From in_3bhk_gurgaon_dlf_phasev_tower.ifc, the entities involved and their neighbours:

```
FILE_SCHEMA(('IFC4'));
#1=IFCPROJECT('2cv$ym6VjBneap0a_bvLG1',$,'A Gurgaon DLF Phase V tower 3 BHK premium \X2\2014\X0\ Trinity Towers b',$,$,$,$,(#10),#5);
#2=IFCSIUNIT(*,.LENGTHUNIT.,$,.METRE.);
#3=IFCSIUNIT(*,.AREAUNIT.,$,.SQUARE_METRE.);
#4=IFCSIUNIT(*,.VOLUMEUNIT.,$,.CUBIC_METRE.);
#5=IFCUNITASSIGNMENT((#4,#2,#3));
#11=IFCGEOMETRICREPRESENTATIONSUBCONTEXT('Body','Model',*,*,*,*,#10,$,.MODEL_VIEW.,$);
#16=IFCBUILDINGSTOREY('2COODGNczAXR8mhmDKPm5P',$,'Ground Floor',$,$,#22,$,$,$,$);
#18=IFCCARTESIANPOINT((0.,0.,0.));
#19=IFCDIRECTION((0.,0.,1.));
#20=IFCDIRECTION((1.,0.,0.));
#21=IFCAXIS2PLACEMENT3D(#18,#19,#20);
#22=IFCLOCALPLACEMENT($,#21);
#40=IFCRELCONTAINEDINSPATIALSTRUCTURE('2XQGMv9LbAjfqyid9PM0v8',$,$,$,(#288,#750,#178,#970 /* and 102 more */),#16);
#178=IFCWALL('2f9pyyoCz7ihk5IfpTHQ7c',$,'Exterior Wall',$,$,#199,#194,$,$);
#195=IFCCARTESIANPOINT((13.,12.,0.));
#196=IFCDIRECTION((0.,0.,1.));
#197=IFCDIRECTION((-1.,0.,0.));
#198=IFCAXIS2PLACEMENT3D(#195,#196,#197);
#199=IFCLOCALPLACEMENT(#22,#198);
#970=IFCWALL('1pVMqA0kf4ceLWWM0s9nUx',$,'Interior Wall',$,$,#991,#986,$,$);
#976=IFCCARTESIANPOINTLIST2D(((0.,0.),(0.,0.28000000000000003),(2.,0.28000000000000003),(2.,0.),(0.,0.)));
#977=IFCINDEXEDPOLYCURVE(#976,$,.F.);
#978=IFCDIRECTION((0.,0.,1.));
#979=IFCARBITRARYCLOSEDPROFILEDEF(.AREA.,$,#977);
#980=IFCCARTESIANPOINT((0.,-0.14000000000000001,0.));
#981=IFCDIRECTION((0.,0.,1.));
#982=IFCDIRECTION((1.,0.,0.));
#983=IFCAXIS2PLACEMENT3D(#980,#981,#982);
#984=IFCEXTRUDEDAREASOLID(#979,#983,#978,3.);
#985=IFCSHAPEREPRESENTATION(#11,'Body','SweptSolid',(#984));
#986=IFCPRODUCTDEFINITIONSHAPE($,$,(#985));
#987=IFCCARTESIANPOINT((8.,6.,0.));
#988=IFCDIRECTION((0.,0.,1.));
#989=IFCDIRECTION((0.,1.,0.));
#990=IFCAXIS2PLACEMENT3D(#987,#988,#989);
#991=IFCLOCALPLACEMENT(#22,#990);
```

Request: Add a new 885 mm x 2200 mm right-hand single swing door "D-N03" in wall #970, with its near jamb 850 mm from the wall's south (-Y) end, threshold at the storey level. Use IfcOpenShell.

```python
import numpy as np
import ifcopenshell
import ifcopenshell.api.feature
import ifcopenshell.api.geometry
import ifcopenshell.api.root
import ifcopenshell.api.spatial
import ifcopenshell.geom
import ifcopenshell.util.element
import ifcopenshell.util.placement
import ifcopenshell.util.representation
import ifcopenshell.util.shape
import ifcopenshell.util.unit

model = ifcopenshell.open("in_3bhk_gurgaon_dlf_phasev_tower.ifc")
unit_scale = ifcopenshell.util.unit.calculate_unit_scale(model)
settings = ifcopenshell.geom.settings()


def volume(element):
    """Net volume in cubic metres, openings subtracted."""
    shape = ifcopenshell.geom.create_shape(settings, element)
    return ifcopenshell.util.shape.get_volume(shape.geometry)


wall = model.by_guid("1pVMqA0kf4ceLWWM0s9nUx")
storey = ifcopenshell.util.element.get_container(wall, ifc_class="IfcBuildingStorey")
context = ifcopenshell.util.representation.get_context(model, "Model", "Body", "MODEL_VIEW")
before = volume(wall)

width, height, from_end, sill = 0.885, 2.2, 0.85, 0.0  # metres

# The wall runs along its own X axis, and the end named is its -X end.
wall_shape = ifcopenshell.geom.create_shape(settings, wall)
x, y, z = ifcopenshell.util.shape.get_vertices(wall_shape.geometry).T
start = x.min() + from_end
face, thickness = float(y.min()), float(y.max() - y.min())
wall_matrix = ifcopenshell.util.placement.get_local_placement(wall.ObjectPlacement)
level = ifcopenshell.util.placement.get_local_placement(storey.ObjectPlacement)[2, 3]


def in_wall(x, y):
    """Placement at x, y metres in the wall's axes, at sill height."""
    matrix = wall_matrix.copy()
    matrix[:, 3] = wall_matrix @ np.array([x / unit_scale, y / unit_scale, 0.0, 1.0])
    matrix[2, 3] = level + sill / unit_scale
    return matrix


# Opening: a box that overshoots both wall faces by 50 mm.
opening = ifcopenshell.api.root.create_entity(model, ifc_class="IfcOpeningElement", predefined_type="OPENING")
box = ifcopenshell.api.geometry.add_wall_representation(
    model, context=context, length=width, height=height, thickness=thickness + 0.1
)
ifcopenshell.api.geometry.assign_representation(model, product=opening, representation=box)
ifcopenshell.api.geometry.edit_object_placement(model, product=opening, matrix=in_wall(start, face - 0.05), is_si=False)
ifcopenshell.api.feature.add_feature(model, feature=opening, element=wall)

door = ifcopenshell.api.root.create_entity(model, ifc_class="IfcDoor", name="D-N03", predefined_type="DOOR")
door.OverallWidth, door.OverallHeight = width / unit_scale, height / unit_scale
door.OperationType = "SINGLE_SWING_RIGHT"
body = ifcopenshell.api.geometry.add_door_representation(
    model,
    context=context,
    overall_width=door.OverallWidth,
    overall_height=door.OverallHeight,
    operation_type="SINGLE_SWING_RIGHT",
    lining_properties={"LiningDepth": thickness / unit_scale, "ThresholdDepth": thickness / unit_scale},
)
ifcopenshell.api.geometry.assign_representation(model, product=door, representation=body)
ifcopenshell.api.spatial.assign_container(model, products=[door], relating_structure=storey)
ifcopenshell.api.feature.add_filling(model, opening=opening, element=door)

# The lining spans the wall, so the door starts at the wall face.
ifcopenshell.api.geometry.edit_object_placement(model, product=door, matrix=in_wall(start, face), is_si=False)

after = volume(wall)

print(f"wall volume {before:.3f} -> {after:.3f} m3")

model.write("in_3bhk_gurgaon_dlf_phasev_tower_v2.ifc")
```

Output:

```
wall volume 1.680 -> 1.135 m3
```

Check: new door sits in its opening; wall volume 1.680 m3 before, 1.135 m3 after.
